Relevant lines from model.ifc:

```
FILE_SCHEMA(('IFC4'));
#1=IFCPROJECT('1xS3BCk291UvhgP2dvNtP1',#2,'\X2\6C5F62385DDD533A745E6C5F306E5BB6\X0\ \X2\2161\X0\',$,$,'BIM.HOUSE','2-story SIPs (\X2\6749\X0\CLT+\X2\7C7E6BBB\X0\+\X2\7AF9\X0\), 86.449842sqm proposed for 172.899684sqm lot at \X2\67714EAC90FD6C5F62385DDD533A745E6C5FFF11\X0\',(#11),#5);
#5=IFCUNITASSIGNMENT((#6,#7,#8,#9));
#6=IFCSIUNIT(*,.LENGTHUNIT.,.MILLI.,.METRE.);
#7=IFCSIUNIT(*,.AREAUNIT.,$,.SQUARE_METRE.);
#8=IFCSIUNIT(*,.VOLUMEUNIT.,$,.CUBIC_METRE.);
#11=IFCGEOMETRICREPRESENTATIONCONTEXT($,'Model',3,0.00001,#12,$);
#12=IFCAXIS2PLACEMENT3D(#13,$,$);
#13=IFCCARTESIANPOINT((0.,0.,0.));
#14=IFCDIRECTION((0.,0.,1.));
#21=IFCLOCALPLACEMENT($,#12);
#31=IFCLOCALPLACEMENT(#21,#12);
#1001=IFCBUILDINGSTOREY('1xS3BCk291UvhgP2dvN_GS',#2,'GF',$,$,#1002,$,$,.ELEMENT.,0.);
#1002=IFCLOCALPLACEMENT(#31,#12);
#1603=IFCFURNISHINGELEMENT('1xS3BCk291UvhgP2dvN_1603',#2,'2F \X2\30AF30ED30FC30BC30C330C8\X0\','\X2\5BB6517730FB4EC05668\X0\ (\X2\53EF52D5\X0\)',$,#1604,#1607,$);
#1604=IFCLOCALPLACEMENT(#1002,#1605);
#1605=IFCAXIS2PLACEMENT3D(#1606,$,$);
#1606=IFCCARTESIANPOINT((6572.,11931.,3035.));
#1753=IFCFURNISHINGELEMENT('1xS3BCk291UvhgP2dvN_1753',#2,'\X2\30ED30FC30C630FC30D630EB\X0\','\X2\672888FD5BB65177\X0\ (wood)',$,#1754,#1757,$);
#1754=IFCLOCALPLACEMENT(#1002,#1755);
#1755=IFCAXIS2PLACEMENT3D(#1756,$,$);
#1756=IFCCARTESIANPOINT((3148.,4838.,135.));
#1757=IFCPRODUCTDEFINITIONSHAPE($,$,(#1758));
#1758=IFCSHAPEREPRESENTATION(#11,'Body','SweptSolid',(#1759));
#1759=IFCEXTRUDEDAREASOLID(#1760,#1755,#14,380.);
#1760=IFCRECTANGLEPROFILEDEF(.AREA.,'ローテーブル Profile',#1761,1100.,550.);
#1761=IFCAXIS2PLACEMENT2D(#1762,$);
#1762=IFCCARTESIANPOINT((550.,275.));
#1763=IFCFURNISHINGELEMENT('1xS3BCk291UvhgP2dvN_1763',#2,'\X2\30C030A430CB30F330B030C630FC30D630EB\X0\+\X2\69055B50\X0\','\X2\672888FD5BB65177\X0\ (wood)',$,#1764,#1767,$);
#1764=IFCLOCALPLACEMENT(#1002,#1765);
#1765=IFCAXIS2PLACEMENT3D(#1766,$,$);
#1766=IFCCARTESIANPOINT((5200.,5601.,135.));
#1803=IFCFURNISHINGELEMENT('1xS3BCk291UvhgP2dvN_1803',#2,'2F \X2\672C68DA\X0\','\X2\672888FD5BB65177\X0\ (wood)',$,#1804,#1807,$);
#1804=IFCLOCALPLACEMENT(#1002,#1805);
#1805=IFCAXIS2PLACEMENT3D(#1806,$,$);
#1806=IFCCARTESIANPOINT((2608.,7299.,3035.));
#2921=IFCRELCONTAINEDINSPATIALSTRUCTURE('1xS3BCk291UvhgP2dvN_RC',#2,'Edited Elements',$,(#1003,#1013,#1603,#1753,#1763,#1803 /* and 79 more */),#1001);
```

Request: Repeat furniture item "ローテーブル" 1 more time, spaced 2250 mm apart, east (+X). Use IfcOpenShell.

```python
import numpy as np
import ifcopenshell
import ifcopenshell.api.geometry
import ifcopenshell.api.root
import ifcopenshell.util.element
import ifcopenshell.util.placement

model = ifcopenshell.open("model.ifc")


def reuse_history(source, copy):
    """copy_class also copies each property set's owner history, people and application; keep the originals."""
    for rel in copy.IsDefinedBy:
        if rel.is_a("IfcRelDefinesByProperties") and (history := rel.RelatingPropertyDefinition.OwnerHistory):
            rel.RelatingPropertyDefinition.OwnerHistory = source.OwnerHistory
            ifcopenshell.util.element.remove_deep2(model, history)


source = model.by_id(1753)
base = ifcopenshell.util.placement.get_local_placement(source.ObjectPlacement)
step = np.array([1.0, 0.0, 0.0]) * 2250.0

for i in range(1, 2):
    copy = ifcopenshell.api.root.copy_class(model, product=source)
    copy.Representation = ifcopenshell.util.element.copy_deep(
        model, source.Representation, exclude=["IfcGeometricRepresentationContext", "IfcRepresentationMap"]
    )
    reuse_history(source, copy)
    matrix = base.copy()
    matrix[:3, 3] += i * step
    print("added at", matrix[:3, 3].round(3) + 0.0)
    ifcopenshell.api.geometry.edit_object_placement(model, product=copy, matrix=matrix, is_si=False)

model.write("model_updated.ifc")
```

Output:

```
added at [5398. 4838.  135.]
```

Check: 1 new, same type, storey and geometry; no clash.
